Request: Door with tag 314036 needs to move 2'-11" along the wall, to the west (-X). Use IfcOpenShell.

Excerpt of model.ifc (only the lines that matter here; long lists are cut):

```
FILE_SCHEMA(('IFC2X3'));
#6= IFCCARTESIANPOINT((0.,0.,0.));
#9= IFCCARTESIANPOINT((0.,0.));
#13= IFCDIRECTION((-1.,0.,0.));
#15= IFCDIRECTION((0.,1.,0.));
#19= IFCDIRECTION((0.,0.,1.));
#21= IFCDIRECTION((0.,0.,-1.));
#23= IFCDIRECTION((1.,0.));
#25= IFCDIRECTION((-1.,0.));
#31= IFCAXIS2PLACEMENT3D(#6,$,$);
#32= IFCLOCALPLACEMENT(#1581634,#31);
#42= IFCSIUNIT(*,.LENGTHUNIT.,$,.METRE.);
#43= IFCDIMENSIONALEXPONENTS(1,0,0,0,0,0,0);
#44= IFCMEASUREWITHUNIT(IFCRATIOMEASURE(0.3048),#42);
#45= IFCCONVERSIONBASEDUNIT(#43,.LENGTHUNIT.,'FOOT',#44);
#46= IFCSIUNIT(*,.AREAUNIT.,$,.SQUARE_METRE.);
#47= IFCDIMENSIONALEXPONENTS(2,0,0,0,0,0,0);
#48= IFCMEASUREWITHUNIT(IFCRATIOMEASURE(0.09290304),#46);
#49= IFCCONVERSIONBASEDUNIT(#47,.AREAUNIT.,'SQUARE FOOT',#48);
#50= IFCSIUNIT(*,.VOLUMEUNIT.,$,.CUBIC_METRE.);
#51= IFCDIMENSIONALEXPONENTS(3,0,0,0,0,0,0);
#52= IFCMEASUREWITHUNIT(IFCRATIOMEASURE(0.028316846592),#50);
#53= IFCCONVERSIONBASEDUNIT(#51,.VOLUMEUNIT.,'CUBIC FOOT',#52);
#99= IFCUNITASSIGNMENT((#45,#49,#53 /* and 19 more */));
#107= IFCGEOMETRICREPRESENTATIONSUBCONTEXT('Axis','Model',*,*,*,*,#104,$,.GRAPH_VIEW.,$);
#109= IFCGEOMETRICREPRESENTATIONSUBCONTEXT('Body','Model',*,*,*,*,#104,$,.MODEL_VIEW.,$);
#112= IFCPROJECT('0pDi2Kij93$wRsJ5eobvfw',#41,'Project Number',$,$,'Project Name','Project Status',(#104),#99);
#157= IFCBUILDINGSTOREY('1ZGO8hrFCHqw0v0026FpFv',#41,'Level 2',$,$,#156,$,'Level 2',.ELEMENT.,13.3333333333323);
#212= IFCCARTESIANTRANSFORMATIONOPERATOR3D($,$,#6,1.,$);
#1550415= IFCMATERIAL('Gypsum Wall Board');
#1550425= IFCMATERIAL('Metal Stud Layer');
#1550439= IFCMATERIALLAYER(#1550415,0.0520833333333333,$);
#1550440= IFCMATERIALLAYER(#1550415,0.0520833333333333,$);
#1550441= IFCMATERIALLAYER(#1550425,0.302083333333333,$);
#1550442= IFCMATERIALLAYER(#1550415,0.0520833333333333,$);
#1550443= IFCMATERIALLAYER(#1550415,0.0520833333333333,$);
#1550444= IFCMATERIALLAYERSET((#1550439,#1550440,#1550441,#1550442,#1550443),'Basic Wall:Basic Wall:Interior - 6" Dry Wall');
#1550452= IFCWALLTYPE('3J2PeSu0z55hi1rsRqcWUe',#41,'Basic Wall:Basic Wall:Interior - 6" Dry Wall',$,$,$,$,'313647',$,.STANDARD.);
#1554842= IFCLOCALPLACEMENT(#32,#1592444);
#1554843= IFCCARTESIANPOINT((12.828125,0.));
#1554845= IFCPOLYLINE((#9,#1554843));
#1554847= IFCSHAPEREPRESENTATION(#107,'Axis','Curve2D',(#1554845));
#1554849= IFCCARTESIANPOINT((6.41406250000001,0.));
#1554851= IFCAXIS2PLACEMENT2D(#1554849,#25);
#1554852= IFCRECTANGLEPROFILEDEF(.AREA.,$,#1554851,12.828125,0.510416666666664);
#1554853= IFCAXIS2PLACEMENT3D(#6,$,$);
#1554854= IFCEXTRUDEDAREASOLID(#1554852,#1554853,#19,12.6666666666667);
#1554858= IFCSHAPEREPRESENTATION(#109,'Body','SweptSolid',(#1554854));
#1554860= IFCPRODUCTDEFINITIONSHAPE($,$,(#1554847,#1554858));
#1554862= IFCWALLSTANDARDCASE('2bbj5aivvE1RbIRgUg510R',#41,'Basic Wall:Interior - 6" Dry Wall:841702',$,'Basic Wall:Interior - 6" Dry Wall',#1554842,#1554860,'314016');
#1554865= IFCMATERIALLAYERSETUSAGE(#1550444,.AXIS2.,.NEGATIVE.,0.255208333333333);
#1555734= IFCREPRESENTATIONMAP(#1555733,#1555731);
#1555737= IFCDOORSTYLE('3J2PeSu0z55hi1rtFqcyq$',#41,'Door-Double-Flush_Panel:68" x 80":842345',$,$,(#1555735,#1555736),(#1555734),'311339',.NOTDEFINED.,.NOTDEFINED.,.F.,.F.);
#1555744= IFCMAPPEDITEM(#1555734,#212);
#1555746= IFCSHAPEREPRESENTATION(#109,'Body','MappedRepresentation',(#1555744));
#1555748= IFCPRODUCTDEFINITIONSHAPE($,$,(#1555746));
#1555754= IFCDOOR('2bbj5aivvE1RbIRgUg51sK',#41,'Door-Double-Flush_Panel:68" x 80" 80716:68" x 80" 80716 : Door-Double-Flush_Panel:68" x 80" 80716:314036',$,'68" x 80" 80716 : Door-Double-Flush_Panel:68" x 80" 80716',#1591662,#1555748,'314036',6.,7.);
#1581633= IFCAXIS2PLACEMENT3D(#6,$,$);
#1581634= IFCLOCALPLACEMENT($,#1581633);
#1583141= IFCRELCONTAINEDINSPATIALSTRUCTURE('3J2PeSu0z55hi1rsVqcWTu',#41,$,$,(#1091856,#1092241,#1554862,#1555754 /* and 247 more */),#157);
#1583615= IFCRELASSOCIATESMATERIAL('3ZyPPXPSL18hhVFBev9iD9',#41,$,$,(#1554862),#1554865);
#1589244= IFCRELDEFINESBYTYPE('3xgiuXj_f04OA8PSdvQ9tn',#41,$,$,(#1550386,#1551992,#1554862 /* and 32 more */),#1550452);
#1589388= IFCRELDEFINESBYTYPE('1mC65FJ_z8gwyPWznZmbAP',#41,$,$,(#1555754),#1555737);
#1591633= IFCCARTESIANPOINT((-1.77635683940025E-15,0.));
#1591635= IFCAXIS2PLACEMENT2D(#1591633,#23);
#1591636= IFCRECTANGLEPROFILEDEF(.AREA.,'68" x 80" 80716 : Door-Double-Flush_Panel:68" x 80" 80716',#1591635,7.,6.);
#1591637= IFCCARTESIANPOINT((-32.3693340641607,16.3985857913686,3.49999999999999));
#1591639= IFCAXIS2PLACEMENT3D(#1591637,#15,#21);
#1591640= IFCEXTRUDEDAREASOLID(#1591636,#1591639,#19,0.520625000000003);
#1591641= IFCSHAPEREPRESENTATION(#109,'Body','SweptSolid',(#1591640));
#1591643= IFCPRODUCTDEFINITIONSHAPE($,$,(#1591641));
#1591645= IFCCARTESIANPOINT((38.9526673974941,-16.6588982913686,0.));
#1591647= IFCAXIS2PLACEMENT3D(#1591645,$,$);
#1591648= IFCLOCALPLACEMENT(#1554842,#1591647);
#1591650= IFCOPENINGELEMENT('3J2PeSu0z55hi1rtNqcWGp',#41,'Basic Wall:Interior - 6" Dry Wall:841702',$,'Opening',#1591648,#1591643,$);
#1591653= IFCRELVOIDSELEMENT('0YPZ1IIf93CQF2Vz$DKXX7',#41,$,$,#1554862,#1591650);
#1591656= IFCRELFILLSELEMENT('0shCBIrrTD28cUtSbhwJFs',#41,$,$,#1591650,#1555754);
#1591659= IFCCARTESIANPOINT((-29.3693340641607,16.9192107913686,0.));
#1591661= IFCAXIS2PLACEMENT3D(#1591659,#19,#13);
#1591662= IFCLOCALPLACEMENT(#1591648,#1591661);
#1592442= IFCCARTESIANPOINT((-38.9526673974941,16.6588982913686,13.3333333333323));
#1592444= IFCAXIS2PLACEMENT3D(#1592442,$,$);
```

```python
import ifcopenshell
import ifcopenshell.api.geometry
import ifcopenshell.util.placement
import ifcopenshell.util.unit

model = ifcopenshell.open("model.ifc")
unit_scale = ifcopenshell.util.unit.calculate_unit_scale(model)

door = model.by_guid("2bbj5aivvE1RbIRgUg51sK")
opening = door.FillsVoids[0].RelatingOpeningElement
wall = opening.VoidsElements[0].RelatingBuildingElement

wall_matrix = ifcopenshell.util.placement.get_local_placement(wall.ObjectPlacement)
shift = wall_matrix[:3, 0] * -35 * 0.0254 / unit_scale
before = ifcopenshell.util.placement.get_local_placement(door.ObjectPlacement)[:3, 3].copy()

# The door is placed relative to its opening, so it follows when the opening moves.
matrix = ifcopenshell.util.placement.get_local_placement(opening.ObjectPlacement)
matrix[:3, 3] += shift
ifcopenshell.api.geometry.edit_object_placement(
    model, product=opening, matrix=matrix, is_si=False, should_transform_children=True
)

after = ifcopenshell.util.placement.get_local_placement(door.ObjectPlacement)[:3, 3]
print("door moved by", (after - before).round(3) + 0.0)

model.write("model_updated.ifc")
```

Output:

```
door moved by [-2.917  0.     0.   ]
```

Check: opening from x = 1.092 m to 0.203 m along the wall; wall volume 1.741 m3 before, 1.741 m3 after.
